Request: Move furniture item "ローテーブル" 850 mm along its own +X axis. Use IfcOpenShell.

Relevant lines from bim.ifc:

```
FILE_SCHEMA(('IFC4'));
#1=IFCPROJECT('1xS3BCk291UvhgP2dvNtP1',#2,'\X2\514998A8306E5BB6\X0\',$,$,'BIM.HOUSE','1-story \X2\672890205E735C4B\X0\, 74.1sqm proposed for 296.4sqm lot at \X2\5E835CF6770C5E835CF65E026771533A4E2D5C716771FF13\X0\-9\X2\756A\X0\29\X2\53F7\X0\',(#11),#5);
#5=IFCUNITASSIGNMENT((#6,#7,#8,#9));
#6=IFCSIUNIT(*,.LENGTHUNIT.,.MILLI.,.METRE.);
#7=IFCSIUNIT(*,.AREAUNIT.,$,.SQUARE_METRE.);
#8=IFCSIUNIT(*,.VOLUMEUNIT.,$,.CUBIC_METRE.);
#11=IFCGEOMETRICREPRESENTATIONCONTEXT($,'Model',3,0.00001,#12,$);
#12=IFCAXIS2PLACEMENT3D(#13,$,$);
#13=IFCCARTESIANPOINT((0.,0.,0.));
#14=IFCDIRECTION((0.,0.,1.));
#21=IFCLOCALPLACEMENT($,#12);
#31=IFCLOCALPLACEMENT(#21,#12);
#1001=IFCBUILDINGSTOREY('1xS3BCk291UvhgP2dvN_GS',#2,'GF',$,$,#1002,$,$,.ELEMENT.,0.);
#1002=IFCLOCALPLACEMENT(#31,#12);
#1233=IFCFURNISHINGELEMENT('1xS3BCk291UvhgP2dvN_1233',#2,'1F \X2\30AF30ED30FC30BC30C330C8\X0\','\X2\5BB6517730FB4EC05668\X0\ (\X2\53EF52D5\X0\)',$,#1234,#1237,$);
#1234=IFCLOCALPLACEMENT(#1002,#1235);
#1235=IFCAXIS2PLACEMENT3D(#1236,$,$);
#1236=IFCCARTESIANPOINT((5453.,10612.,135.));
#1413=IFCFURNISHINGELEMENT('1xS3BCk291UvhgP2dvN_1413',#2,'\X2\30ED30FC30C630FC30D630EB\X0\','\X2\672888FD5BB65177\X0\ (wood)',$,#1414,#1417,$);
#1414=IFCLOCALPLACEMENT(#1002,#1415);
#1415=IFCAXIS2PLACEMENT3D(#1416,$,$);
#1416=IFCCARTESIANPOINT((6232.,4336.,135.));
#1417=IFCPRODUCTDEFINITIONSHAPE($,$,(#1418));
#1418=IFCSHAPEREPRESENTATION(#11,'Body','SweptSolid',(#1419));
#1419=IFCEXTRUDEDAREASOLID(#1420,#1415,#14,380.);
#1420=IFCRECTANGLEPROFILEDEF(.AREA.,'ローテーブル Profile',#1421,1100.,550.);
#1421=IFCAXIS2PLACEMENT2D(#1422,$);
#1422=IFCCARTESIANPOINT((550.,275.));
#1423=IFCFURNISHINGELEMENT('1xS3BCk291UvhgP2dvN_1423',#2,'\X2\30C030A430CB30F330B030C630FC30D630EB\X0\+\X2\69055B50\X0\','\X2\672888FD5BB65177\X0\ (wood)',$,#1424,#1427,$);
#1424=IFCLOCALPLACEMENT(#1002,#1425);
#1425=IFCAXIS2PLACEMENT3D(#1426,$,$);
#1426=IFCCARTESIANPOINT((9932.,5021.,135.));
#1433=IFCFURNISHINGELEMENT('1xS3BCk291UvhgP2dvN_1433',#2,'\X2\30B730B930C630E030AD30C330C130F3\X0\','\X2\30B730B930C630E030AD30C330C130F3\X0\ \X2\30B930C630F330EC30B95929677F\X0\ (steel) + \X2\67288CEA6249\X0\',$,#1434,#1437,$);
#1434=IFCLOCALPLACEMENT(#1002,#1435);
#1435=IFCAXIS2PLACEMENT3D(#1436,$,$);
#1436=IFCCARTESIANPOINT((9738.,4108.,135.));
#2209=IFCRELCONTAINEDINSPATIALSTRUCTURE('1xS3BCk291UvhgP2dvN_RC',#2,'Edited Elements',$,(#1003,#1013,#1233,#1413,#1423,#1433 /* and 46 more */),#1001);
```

```python
import ifcopenshell
import ifcopenshell.api.geometry
import ifcopenshell.util.placement

model = ifcopenshell.open("bim.ifc")

item = model.by_guid("1xS3BCk291UvhgP2dvN_1413")
matrix = ifcopenshell.util.placement.get_local_placement(item.ObjectPlacement)
matrix[:3, 3] += matrix[:3, 0] * 850.0
ifcopenshell.api.geometry.edit_object_placement(model, product=item, matrix=matrix, is_si=False)

print(ifcopenshell.util.placement.get_local_placement(item.ObjectPlacement).round(3) + 0.0)

model.write("bim_rev.ifc")
```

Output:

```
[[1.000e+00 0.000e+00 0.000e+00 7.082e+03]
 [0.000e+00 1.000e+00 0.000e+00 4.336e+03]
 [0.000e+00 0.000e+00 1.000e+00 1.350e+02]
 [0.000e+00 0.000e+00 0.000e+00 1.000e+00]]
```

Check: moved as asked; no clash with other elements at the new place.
